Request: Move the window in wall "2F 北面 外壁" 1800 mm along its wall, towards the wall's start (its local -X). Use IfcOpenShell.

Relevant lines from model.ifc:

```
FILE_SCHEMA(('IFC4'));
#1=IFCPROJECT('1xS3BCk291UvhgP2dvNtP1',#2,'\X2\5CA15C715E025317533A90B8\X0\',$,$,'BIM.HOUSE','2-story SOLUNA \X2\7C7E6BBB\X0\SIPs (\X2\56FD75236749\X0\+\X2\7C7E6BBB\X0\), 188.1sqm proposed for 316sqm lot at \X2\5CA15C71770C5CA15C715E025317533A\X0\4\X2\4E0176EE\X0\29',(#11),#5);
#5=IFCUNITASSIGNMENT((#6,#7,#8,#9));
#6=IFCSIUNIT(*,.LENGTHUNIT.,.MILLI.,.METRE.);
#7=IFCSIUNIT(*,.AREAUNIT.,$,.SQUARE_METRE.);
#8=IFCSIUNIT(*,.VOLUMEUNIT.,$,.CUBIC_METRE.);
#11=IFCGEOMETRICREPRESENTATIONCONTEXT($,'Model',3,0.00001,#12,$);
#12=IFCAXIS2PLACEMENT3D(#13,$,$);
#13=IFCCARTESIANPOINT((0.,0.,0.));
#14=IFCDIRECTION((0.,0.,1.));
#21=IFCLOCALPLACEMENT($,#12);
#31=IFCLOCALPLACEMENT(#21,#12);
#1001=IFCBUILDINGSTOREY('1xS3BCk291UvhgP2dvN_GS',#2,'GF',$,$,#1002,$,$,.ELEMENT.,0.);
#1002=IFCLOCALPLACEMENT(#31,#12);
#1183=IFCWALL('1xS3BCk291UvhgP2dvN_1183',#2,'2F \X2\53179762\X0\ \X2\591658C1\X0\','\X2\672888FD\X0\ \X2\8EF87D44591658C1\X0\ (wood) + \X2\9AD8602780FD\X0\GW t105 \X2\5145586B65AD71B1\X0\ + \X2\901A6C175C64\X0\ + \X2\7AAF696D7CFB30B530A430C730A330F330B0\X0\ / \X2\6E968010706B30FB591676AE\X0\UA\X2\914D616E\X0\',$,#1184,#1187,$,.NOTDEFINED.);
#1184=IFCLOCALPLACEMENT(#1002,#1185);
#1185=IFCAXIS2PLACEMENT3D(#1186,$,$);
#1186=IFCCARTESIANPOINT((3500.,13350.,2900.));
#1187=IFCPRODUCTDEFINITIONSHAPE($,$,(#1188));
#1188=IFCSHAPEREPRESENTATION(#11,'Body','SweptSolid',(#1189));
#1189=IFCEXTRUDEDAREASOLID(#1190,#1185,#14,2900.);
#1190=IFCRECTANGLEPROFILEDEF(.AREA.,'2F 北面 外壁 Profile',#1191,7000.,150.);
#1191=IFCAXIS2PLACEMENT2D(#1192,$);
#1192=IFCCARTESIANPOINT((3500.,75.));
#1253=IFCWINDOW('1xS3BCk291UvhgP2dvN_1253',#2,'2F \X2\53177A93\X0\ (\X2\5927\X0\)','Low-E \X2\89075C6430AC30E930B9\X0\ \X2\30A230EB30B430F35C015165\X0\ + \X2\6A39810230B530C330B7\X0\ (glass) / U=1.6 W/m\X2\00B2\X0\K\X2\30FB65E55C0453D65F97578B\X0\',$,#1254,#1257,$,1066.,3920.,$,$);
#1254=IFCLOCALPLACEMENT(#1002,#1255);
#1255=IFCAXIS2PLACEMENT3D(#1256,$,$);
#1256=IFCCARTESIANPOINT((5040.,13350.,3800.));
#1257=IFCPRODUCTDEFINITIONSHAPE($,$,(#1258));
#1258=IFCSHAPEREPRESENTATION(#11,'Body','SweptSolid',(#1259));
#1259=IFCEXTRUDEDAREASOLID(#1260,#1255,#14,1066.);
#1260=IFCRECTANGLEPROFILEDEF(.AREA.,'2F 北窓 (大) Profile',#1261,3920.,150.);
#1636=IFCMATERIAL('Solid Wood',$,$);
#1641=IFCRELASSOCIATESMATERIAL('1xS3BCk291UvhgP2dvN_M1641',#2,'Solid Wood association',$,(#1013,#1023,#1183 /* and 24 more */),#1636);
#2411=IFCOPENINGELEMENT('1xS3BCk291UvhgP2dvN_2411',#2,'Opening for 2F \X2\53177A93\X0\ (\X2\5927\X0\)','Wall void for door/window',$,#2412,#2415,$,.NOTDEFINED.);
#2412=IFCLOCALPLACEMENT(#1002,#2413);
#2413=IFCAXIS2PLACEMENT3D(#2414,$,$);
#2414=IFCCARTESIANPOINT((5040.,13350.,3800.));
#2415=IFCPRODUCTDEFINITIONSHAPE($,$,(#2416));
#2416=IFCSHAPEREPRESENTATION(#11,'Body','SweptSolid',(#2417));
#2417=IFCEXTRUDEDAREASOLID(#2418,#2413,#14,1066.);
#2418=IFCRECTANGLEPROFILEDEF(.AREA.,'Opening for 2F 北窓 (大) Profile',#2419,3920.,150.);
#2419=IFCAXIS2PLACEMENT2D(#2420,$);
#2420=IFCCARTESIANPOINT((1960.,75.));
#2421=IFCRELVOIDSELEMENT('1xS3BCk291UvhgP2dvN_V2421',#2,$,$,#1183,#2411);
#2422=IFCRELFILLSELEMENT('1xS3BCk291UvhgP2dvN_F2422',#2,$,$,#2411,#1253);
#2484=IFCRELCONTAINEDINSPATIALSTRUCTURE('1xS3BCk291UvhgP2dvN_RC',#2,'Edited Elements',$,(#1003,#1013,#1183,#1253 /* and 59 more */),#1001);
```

```python
import ifcopenshell
import ifcopenshell.api.geometry
import ifcopenshell.util.placement
import ifcopenshell.util.unit

model = ifcopenshell.open("model.ifc")
unit_scale = ifcopenshell.util.unit.calculate_unit_scale(model)

window = model.by_guid("1xS3BCk291UvhgP2dvN_1253")
opening = window.FillsVoids[0].RelatingOpeningElement
wall = opening.VoidsElements[0].RelatingBuildingElement

wall_matrix = ifcopenshell.util.placement.get_local_placement(wall.ObjectPlacement)
shift = wall_matrix[:3, 0] * -1.8 / unit_scale
before = ifcopenshell.util.placement.get_local_placement(window.ObjectPlacement)[:3, 3].copy()

# The window is not placed relative to its opening, so move both.
for product in (opening, window):
    matrix = ifcopenshell.util.placement.get_local_placement(product.ObjectPlacement)
    matrix[:3, 3] += shift
    ifcopenshell.api.geometry.edit_object_placement(model, product=product, matrix=matrix, is_si=False)

after = ifcopenshell.util.placement.get_local_placement(window.ObjectPlacement)[:3, 3]
print("window moved by", (after - before).round(3) + 0.0)

model.write("model-out.ifc")
```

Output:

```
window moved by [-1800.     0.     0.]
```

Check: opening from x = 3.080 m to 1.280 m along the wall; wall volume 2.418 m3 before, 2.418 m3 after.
